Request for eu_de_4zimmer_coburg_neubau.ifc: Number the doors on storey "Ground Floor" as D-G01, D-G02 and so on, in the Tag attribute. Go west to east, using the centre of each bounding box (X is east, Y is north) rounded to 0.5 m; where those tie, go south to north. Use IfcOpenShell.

First a look at what the model holds.

```python
import ifcopenshell
import ifcopenshell.util.element
import ifcopenshell.util.placement

model = ifcopenshell.open("eu_de_4zimmer_coburg_neubau.ifc")
print(model.schema)
storey = next(s for s in model.by_type("IfcBuildingStorey") if s.Name == "Ground Floor")
doors = [e for e in ifcopenshell.util.element.get_decomposition(storey) if e.is_a("IfcDoor")]
for e in sorted(doors, key=lambda e: e.id()):
    origin = ifcopenshell.util.placement.get_local_placement(e.ObjectPlacement)[:3, 3]
    print(e.id(), e.Tag, e.Name, origin.round(2) + 0.0, sep=" | ")
```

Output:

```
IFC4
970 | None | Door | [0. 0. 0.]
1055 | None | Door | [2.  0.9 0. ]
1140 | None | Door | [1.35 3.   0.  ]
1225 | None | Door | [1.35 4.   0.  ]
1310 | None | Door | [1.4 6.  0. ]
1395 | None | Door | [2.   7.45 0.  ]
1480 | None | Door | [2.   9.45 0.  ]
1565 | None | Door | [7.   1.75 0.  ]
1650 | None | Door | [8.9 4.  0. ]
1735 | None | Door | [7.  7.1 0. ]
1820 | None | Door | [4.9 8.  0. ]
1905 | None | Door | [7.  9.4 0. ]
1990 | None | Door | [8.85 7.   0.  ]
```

```python
import ifcopenshell
import ifcopenshell.geom
import ifcopenshell.util.element
import ifcopenshell.util.shape

model = ifcopenshell.open("eu_de_4zimmer_coburg_neubau.ifc")
settings = ifcopenshell.geom.settings()
settings.set("use-world-coords", True)


def centre(element):
    shape = ifcopenshell.geom.create_shape(settings, element)
    return ifcopenshell.util.shape.get_bbox_centroid(shape.geometry)


storey = next(s for s in model.by_type("IfcBuildingStorey") if s.Name == "Ground Floor")
doors = [e for e in ifcopenshell.util.element.get_decomposition(storey) if e.is_a("IfcDoor")]

# Insertion points can sit at a corner or the storey origin, so sort by the geometry (in metres).
centres = {e: centre(e) for e in doors}
doors.sort(key=lambda e: (round(centres[e][0] / 0.5), centres[e][1]))

for i, e in enumerate(doors, start=1):
    number = f"D-G{i:02d}"
    e.Tag = number
    print(e.id(), number)

model.write("eu_de_4zimmer_coburg_neubau-out.ifc")
```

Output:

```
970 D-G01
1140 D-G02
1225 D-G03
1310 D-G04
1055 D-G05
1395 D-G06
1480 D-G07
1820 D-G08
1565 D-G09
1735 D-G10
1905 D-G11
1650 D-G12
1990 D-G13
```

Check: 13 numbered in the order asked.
